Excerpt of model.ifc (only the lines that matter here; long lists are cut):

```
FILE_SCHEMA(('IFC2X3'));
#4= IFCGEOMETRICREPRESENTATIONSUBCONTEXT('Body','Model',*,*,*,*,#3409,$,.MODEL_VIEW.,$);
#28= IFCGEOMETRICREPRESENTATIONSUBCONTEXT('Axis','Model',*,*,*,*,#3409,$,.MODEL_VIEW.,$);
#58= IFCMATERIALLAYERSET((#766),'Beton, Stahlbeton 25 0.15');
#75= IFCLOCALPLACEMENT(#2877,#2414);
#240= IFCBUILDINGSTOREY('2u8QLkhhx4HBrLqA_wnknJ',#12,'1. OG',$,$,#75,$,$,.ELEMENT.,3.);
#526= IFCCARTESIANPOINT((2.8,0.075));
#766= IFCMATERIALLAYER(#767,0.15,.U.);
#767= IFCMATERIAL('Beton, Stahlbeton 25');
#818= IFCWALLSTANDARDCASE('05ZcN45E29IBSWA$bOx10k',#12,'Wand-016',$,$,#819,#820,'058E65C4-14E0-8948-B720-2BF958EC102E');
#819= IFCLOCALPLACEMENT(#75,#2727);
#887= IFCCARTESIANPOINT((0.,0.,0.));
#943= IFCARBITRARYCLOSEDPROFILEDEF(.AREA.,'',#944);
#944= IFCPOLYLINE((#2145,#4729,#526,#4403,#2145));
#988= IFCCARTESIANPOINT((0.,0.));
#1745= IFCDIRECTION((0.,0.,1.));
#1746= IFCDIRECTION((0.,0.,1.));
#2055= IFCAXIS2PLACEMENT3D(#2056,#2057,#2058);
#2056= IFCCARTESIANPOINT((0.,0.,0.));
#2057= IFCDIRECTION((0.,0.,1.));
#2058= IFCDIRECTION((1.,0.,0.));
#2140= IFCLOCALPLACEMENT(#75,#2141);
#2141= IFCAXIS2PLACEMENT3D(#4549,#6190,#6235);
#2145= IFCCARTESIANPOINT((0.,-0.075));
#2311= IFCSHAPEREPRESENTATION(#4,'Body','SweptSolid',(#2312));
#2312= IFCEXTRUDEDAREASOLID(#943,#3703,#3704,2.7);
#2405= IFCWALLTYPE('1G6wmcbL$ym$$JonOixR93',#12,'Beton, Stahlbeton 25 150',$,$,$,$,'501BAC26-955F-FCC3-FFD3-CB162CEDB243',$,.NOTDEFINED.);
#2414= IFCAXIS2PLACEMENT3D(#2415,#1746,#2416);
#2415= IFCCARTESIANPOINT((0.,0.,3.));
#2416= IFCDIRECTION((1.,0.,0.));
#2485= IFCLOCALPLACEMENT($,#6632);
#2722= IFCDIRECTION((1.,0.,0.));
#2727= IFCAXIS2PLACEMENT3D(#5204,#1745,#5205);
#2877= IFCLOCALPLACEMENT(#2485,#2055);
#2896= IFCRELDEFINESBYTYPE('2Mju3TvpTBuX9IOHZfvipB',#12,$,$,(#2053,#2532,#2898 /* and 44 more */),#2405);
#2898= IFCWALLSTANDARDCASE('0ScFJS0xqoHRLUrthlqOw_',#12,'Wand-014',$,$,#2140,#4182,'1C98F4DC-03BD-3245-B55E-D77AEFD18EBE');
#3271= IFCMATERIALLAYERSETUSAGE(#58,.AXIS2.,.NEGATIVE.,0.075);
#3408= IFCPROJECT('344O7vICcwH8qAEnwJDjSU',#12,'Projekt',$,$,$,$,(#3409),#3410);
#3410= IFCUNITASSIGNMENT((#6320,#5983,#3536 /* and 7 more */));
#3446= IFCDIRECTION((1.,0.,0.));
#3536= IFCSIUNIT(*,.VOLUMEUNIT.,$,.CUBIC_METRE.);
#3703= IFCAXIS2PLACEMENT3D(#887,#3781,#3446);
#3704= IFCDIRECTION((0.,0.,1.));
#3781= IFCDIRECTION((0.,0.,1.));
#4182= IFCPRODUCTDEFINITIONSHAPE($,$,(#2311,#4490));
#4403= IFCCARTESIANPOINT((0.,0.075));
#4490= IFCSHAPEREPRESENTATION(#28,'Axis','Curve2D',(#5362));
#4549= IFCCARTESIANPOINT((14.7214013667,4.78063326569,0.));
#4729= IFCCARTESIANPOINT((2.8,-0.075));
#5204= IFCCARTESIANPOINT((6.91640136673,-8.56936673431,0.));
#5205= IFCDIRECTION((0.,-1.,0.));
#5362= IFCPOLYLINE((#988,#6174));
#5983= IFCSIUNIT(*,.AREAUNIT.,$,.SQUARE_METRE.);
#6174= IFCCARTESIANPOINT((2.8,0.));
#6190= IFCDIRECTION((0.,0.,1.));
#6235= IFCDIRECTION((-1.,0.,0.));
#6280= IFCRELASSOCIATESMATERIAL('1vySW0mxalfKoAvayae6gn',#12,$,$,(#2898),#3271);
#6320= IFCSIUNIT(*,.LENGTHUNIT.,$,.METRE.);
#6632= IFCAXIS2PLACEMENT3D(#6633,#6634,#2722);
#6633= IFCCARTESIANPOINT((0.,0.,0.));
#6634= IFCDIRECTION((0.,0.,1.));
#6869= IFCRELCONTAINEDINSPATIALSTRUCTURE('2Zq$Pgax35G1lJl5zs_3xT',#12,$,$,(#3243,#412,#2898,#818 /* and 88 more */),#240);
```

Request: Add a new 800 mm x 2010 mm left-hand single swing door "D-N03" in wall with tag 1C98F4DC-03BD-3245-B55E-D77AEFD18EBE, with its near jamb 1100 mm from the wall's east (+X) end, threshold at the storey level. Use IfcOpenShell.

```python
import numpy as np
import ifcopenshell
import ifcopenshell.api.feature
import ifcopenshell.api.geometry
import ifcopenshell.api.root
import ifcopenshell.api.spatial
import ifcopenshell.api.type
import ifcopenshell.geom
import ifcopenshell.util.element
import ifcopenshell.util.placement
import ifcopenshell.util.representation
import ifcopenshell.util.shape
import ifcopenshell.util.unit

model = ifcopenshell.open("model.ifc")
unit_scale = ifcopenshell.util.unit.calculate_unit_scale(model)
settings = ifcopenshell.geom.settings()


def volume(element):
    """Net volume in cubic metres, openings subtracted."""
    shape = ifcopenshell.geom.create_shape(settings, element)
    return ifcopenshell.util.shape.get_volume(shape.geometry)


wall = model.by_id(2898)
storey = ifcopenshell.util.element.get_container(wall, ifc_class="IfcBuildingStorey")
context = ifcopenshell.util.representation.get_context(model, "Model", "Body", "MODEL_VIEW")
before = volume(wall)

width, height, from_end, sill = 0.8, 2.01, 1.1, 0.0  # metres

# The wall runs along its own X axis, and the end named is its -X end.
wall_shape = ifcopenshell.geom.create_shape(settings, wall)
x, y, z = ifcopenshell.util.shape.get_vertices(wall_shape.geometry).T
start = x.min() + from_end
face, thickness = float(y.min()), float(y.max() - y.min())
wall_matrix = ifcopenshell.util.placement.get_local_placement(wall.ObjectPlacement)
level = ifcopenshell.util.placement.get_local_placement(storey.ObjectPlacement)[2, 3]


def in_wall(x, y):
    """Placement at x, y metres in the wall's axes, at sill height."""
    matrix = wall_matrix.copy()
    matrix[:, 3] = wall_matrix @ np.array([x / unit_scale, y / unit_scale, 0.0, 1.0])
    matrix[2, 3] = level + sill / unit_scale
    return matrix


# Opening: a box that overshoots both wall faces by 50 mm.
opening = ifcopenshell.api.root.create_entity(model, ifc_class="IfcOpeningElement")
box = ifcopenshell.api.geometry.add_wall_representation(
    model, context=context, length=width, height=height, thickness=thickness + 0.1
)
ifcopenshell.api.geometry.assign_representation(model, product=opening, representation=box)
ifcopenshell.api.geometry.edit_object_placement(model, product=opening, matrix=in_wall(start, face - 0.05), is_si=False)
ifcopenshell.api.feature.add_feature(model, feature=opening, element=wall)

door = ifcopenshell.api.root.create_entity(model, ifc_class="IfcDoor", name="D-N03")
door.OverallWidth, door.OverallHeight = width / unit_scale, height / unit_scale
body = ifcopenshell.api.geometry.add_door_representation(
    model,
    context=context,
    overall_width=door.OverallWidth,
    overall_height=door.OverallHeight,
    operation_type="SINGLE_SWING_LEFT",
    lining_properties={"LiningDepth": thickness / unit_scale, "ThresholdDepth": thickness / unit_scale},
)
ifcopenshell.api.geometry.assign_representation(model, product=door, representation=body)
ifcopenshell.api.spatial.assign_container(model, products=[door], relating_structure=storey)
fills = ifcopenshell.api.feature.add_filling(model, opening=opening, element=door)
fills.OwnerHistory = door.OwnerHistory  # required in IFC2X3

# IFC2X3 keeps the operation on the door style.
style = ifcopenshell.api.root.create_entity(model, ifc_class="IfcDoorStyle", name="D-N03")
style.OperationType, style.ConstructionType = "SINGLE_SWING_LEFT", "NOTDEFINED"
style.ParameterTakesPrecedence = style.Sizeable = False
ifcopenshell.api.type.assign_type(model, related_objects=[door], relating_type=style)

# The lining spans the wall, so the door starts at the wall face.
ifcopenshell.api.geometry.edit_object_placement(model, product=door, matrix=in_wall(start, face), is_si=False)

after = volume(wall)

print(f"wall volume {before:.3f} -> {after:.3f} m3")

model.write("model_updated.ifc")
```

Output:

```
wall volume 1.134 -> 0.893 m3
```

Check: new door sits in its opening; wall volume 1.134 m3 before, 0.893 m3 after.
